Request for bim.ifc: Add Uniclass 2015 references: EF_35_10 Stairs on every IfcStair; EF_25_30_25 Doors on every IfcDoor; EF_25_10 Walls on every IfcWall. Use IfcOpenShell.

First a look at what the model holds.

```python
import ifcopenshell

model = ifcopenshell.open("bim.ifc")
print(model.schema)
print("classifications:", [c.Name for c in model.by_type("IfcClassification")])
for ifc_class in ("IfcDoor", "IfcRoof", "IfcStair", "IfcWall", "IfcWindow"):
    print(ifc_class, len(model.by_type(ifc_class)))
```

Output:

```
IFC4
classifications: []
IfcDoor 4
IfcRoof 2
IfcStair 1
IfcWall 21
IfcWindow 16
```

```python
import ifcopenshell
import ifcopenshell.api.classification

model = ifcopenshell.open("bim.ifc")

system = ifcopenshell.api.classification.add_classification(model, classification="Uniclass 2015")

codes = {
    "IfcStair": ("EF_35_10", "Stairs"),
    "IfcDoor": ("EF_25_30_25", "Doors"),
    "IfcWall": ("EF_25_10", "Walls"),
}
for ifc_class, (code, name) in codes.items():
    products = model.by_type(ifc_class)
    ifcopenshell.api.classification.add_reference(
        model, products=products, classification=system, identification=code, name=name
    )
    print(code, len(products))

model.write("bim-out.ifc")
```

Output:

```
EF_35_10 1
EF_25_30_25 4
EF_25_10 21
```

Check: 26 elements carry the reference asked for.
